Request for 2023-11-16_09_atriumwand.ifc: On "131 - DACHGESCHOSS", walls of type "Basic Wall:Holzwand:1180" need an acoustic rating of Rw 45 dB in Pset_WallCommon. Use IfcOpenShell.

First a look at what the model holds.

```python
import ifcopenshell
import ifcopenshell.util.element

model = ifcopenshell.open("2023-11-16_09_atriumwand.ifc")
print(model.schema)
storey = next(s for s in model.by_type("IfcBuildingStorey") if s.Name == "131 - DACHGESCHOSS")
walls = [e for e in ifcopenshell.util.element.get_decomposition(storey) if e.is_a("IfcWall")]
seen = {}
for e in walls:
    element_type = ifcopenshell.util.element.get_type(e)
    key = (element_type.Name if element_type != e and element_type else None, ifcopenshell.util.element.get_pset(e, "Pset_WallCommon", "AcousticRating"))
    seen[key] = seen.get(key, 0) + 1
for (name, value), count in sorted(seen.items(), key=str):
    print(count, "x", name, "|", value)
```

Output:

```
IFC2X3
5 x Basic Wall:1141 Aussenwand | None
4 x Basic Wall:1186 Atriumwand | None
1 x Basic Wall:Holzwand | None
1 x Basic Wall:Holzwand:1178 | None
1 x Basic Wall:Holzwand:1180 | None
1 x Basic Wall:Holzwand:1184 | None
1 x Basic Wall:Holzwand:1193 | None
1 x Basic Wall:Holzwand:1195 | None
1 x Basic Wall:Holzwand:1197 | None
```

```python
import ifcopenshell
import ifcopenshell.api.pset
import ifcopenshell.util.element

model = ifcopenshell.open("2023-11-16_09_atriumwand.ifc")

storey = next(s for s in model.by_type("IfcBuildingStorey") if s.Name == "131 - DACHGESCHOSS")
walls = [e for e in ifcopenshell.util.element.get_decomposition(storey) if e.is_a("IfcWall")]

count = 0
for e in walls:
    element_type = ifcopenshell.util.element.get_type(e)
    if element_type in (None, e) or element_type.Name != "Basic Wall:Holzwand:1180":
        continue
    # add_pset returns the element's existing set when there is one.
    pset = ifcopenshell.api.pset.add_pset(model, product=e, name="Pset_WallCommon")
    ifcopenshell.api.pset.edit_pset(model, pset=pset, properties={"AcousticRating": "Rw 45 dB"})
    count += 1

print(count, "walls updated")

model.write("2023-11-16_09_atriumwand_rev.ifc")
```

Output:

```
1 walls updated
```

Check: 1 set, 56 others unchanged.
